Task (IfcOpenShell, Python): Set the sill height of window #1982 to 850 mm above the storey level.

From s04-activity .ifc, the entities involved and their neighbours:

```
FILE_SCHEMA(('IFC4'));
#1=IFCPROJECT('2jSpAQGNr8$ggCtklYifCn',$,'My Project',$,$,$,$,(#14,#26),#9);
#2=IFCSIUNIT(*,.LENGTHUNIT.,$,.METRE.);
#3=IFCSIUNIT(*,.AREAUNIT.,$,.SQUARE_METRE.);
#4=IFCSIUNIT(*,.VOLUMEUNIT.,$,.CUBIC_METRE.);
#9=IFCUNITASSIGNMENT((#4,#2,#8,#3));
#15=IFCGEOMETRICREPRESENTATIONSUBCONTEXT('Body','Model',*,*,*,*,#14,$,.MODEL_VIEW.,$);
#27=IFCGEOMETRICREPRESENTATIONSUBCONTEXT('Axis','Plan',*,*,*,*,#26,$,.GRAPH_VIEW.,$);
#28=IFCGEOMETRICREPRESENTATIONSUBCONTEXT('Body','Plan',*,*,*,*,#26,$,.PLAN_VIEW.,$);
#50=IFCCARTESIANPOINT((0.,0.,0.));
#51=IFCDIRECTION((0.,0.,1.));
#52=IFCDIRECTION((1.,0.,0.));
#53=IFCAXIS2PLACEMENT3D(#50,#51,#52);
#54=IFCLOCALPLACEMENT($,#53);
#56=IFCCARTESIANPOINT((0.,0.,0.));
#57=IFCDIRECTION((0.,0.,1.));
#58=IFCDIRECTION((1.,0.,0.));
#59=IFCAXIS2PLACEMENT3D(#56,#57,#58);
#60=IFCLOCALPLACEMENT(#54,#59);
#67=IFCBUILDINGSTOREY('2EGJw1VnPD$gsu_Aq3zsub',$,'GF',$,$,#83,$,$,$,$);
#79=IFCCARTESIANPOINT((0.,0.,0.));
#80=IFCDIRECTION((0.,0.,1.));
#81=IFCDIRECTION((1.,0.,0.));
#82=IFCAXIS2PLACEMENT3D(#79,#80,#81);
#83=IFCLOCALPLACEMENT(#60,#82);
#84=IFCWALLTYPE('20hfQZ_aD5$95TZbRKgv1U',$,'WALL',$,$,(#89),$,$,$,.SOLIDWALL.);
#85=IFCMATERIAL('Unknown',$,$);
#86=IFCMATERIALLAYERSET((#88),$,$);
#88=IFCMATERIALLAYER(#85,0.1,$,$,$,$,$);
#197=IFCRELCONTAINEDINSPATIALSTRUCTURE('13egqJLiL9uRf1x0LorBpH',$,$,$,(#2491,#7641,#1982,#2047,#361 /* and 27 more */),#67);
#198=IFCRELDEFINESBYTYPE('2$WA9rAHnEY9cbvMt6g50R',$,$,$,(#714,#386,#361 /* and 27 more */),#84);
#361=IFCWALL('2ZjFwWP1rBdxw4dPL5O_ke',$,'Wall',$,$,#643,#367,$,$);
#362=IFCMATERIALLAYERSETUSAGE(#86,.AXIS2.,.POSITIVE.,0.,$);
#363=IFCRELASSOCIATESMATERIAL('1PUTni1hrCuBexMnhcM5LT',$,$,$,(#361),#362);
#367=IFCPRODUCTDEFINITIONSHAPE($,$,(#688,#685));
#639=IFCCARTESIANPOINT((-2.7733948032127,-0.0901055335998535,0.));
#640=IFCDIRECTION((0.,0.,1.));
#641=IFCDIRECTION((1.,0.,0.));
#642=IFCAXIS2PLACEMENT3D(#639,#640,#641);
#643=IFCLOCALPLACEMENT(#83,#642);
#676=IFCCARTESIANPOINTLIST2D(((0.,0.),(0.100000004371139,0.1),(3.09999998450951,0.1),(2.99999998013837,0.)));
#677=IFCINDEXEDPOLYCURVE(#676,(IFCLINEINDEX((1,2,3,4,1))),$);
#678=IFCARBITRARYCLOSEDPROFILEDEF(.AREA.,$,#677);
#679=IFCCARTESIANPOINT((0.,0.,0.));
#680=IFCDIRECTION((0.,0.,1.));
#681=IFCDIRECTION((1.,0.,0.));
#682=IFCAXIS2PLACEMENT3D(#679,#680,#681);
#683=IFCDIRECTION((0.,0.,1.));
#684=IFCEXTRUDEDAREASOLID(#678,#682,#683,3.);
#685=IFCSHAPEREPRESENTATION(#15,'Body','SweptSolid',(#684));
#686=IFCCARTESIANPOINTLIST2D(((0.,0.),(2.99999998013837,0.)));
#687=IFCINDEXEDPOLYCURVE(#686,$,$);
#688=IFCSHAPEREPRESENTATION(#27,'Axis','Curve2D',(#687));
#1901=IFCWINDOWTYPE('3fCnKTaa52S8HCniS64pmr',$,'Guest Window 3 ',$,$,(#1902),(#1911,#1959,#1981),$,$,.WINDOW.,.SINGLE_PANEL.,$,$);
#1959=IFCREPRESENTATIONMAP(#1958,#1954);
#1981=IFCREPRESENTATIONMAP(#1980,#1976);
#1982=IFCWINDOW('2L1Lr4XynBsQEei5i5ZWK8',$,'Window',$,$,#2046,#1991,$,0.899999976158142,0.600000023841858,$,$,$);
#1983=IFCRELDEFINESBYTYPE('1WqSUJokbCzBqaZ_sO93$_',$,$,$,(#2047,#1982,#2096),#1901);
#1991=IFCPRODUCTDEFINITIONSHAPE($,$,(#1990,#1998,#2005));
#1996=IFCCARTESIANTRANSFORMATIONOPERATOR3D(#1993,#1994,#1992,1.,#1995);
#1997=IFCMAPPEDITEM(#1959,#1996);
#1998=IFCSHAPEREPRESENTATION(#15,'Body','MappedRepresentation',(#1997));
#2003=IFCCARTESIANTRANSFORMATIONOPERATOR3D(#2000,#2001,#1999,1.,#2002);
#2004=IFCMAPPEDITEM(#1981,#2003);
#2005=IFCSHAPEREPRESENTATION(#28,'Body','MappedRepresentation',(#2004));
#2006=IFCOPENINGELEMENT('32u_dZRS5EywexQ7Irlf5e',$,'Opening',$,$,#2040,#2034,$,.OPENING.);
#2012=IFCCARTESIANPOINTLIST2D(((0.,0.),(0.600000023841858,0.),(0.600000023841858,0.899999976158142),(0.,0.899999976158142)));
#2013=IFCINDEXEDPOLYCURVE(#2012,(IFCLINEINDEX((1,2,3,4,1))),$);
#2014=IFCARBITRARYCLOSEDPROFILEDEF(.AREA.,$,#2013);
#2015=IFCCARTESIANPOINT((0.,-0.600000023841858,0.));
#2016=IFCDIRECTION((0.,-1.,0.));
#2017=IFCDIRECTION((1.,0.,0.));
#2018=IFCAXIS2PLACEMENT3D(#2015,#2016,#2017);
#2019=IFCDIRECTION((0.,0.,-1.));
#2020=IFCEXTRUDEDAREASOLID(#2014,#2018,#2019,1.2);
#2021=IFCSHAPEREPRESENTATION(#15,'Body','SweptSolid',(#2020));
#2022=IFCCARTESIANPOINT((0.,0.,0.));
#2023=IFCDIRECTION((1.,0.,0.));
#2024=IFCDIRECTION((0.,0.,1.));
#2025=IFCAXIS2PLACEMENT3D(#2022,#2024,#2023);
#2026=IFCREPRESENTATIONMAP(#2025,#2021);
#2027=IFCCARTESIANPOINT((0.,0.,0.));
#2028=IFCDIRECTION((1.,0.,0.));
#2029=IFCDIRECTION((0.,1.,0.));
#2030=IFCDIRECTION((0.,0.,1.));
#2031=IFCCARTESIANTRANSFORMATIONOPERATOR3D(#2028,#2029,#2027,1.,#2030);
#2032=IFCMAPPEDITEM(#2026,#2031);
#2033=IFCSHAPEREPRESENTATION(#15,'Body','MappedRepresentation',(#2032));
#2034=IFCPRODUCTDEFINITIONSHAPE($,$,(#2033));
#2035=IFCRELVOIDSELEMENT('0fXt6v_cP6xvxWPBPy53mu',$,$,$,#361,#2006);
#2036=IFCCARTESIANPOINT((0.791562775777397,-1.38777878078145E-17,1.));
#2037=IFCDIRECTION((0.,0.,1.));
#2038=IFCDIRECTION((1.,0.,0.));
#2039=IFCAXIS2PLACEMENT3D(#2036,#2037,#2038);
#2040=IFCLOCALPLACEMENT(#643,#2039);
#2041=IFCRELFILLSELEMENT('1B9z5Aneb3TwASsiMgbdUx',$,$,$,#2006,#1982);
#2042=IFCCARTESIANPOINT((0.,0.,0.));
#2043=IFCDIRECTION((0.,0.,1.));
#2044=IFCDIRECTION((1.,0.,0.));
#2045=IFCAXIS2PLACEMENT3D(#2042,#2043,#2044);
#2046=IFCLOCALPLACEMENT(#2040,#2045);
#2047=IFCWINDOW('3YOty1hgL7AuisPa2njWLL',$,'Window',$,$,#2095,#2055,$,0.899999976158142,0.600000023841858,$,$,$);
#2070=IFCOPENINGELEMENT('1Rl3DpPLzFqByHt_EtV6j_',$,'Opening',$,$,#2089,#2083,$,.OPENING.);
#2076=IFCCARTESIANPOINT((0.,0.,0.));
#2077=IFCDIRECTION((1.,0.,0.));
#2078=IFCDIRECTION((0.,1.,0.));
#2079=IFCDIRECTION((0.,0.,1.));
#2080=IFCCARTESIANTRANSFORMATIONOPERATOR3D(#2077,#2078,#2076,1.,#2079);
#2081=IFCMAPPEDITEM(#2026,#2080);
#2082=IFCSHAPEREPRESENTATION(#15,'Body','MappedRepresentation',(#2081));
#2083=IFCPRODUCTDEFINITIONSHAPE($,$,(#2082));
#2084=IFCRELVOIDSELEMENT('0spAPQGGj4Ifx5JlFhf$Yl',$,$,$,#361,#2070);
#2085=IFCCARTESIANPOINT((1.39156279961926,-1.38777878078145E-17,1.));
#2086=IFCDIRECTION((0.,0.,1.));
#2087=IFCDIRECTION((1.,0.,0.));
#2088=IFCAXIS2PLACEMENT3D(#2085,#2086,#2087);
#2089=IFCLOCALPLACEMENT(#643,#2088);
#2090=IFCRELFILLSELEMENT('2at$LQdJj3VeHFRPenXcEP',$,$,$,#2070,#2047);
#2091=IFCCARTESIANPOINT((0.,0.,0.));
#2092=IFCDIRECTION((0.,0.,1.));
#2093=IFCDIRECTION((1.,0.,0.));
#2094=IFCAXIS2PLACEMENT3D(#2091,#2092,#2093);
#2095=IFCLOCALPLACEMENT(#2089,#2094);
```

```python
import numpy as np
import ifcopenshell
import ifcopenshell.api.geometry
import ifcopenshell.geom
import ifcopenshell.util.element
import ifcopenshell.util.placement
import ifcopenshell.util.shape
import ifcopenshell.util.unit

model = ifcopenshell.open("s04-activity .ifc")
unit_scale = ifcopenshell.util.unit.calculate_unit_scale(model)

window = model.by_id(1982)
opening = window.FillsVoids[0].RelatingOpeningElement
storey = ifcopenshell.util.element.get_container(window, ifc_class="IfcBuildingStorey")
level = ifcopenshell.util.placement.get_local_placement(storey.ObjectPlacement)[2, 3]

# The opening's origin need not be at the sill, so measure its lowest point.
shape = ifcopenshell.geom.create_shape(ifcopenshell.geom.settings(), opening)
bottom = ifcopenshell.util.shape.get_shape_bottom_elevation(shape, shape.geometry) / unit_scale
dz = level + 0.85 - bottom

shift = np.array([0.0, 0.0, dz])
# The window is placed relative to its opening, so it follows when the opening moves.
matrix = ifcopenshell.util.placement.get_local_placement(opening.ObjectPlacement)
matrix[:3, 3] += shift
ifcopenshell.api.geometry.edit_object_placement(
    model, product=opening, matrix=matrix, is_si=False, should_transform_children=True
)

print(f"moved by {dz * unit_scale:+.3f} m")

model.write("s04-activity -out.ifc")
```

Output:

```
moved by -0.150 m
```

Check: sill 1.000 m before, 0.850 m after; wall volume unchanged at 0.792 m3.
